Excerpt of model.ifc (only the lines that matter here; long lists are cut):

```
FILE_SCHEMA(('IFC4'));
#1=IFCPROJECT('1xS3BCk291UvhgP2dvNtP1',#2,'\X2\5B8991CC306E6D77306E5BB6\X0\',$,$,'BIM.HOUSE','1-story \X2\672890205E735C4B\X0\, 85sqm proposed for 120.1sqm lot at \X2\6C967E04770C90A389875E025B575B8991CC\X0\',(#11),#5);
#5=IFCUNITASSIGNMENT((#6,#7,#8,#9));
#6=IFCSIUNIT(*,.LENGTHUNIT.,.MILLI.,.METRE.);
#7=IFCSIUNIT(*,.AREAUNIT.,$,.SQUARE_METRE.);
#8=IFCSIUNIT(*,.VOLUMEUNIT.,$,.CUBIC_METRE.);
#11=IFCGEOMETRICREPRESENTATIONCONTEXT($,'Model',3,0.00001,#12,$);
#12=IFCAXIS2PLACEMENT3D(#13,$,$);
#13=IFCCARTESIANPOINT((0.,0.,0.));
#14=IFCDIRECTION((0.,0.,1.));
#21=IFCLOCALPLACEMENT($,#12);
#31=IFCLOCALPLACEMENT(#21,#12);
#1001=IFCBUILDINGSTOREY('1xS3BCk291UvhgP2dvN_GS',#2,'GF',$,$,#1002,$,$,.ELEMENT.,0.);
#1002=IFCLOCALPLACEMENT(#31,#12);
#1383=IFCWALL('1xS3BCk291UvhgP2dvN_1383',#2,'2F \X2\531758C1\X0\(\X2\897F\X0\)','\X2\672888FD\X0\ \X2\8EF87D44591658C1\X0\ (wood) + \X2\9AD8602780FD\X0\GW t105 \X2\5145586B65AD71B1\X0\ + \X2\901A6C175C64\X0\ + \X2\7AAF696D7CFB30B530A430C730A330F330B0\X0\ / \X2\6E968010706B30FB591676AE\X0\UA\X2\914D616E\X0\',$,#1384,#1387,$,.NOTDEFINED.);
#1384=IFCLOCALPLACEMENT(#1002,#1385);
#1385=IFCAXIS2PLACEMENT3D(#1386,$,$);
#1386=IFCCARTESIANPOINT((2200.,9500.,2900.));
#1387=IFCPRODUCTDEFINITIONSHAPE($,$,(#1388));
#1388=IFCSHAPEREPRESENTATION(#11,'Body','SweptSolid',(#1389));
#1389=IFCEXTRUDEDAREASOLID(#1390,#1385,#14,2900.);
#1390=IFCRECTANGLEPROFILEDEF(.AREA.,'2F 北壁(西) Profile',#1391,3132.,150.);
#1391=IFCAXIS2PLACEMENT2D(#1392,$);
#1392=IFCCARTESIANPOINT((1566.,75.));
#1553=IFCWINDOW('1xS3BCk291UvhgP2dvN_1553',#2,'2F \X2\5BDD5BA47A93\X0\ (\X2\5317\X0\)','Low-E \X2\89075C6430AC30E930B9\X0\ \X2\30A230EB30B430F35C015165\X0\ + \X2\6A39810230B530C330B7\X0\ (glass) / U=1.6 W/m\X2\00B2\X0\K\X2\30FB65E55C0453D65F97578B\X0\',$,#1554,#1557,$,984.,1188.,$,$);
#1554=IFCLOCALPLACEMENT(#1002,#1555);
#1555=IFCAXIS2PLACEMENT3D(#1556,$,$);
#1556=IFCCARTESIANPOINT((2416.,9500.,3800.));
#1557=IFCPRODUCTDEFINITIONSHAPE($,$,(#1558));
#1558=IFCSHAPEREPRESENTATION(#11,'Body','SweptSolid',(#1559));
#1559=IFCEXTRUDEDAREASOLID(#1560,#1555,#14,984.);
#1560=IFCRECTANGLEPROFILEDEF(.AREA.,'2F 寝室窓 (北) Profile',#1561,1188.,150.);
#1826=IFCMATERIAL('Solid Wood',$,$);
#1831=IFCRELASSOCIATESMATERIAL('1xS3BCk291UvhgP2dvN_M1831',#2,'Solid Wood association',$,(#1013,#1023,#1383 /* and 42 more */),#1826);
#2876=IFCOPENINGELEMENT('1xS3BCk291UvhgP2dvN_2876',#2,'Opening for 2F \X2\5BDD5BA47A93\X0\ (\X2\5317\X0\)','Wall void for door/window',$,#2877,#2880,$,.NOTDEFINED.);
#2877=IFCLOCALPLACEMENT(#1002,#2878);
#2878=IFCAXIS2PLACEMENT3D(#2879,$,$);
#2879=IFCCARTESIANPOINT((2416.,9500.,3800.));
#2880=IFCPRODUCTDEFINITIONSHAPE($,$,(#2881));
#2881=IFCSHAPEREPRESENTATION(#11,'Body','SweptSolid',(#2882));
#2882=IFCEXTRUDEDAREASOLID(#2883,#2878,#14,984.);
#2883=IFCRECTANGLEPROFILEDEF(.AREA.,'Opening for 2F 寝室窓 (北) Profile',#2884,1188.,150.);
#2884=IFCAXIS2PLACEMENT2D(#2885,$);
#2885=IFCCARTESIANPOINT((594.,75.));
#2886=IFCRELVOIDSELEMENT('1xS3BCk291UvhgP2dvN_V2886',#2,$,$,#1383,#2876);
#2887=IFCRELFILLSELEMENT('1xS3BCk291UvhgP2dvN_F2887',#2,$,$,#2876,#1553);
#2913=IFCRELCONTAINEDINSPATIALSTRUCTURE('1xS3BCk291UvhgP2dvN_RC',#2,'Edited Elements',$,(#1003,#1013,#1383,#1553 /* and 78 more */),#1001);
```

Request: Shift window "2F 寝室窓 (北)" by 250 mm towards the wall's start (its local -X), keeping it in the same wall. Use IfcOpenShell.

```python
import ifcopenshell
import ifcopenshell.api.geometry
import ifcopenshell.util.placement
import ifcopenshell.util.unit

model = ifcopenshell.open("model.ifc")
unit_scale = ifcopenshell.util.unit.calculate_unit_scale(model)

window = model.by_id(1553)
opening = window.FillsVoids[0].RelatingOpeningElement
wall = opening.VoidsElements[0].RelatingBuildingElement

wall_matrix = ifcopenshell.util.placement.get_local_placement(wall.ObjectPlacement)
shift = wall_matrix[:3, 0] * -0.25 / unit_scale
before = ifcopenshell.util.placement.get_local_placement(window.ObjectPlacement)[:3, 3].copy()

# The window is not placed relative to its opening, so move both.
for product in (opening, window):
    matrix = ifcopenshell.util.placement.get_local_placement(product.ObjectPlacement)
    matrix[:3, 3] += shift
    ifcopenshell.api.geometry.edit_object_placement(model, product=product, matrix=matrix, is_si=False)

after = ifcopenshell.util.placement.get_local_placement(window.ObjectPlacement)[:3, 3]
print("window moved by", (after - before).round(3) + 0.0)

model.write("model_updated.ifc")
```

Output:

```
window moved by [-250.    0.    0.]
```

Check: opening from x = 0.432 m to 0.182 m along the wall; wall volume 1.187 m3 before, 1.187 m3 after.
